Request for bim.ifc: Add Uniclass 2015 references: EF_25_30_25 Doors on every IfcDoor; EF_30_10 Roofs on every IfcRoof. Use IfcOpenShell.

First a look at what the model holds.

```python
import ifcopenshell

model = ifcopenshell.open("bim.ifc")
print(model.schema)
print("classifications:", [c.Name for c in model.by_type("IfcClassification")])
for ifc_class in ("IfcDoor", "IfcRoof", "IfcStair", "IfcWall", "IfcWindow"):
    print(ifc_class, len(model.by_type(ifc_class)))
```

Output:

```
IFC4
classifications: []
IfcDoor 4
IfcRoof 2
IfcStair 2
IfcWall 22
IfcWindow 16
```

```python
import ifcopenshell
import ifcopenshell.api.classification

model = ifcopenshell.open("bim.ifc")

system = ifcopenshell.api.classification.add_classification(model, classification="Uniclass 2015")

codes = {
    "IfcDoor": ("EF_25_30_25", "Doors"),
    "IfcRoof": ("EF_30_10", "Roofs"),
}
for ifc_class, (code, name) in codes.items():
    products = model.by_type(ifc_class)
    ifcopenshell.api.classification.add_reference(
        model, products=products, classification=system, identification=code, name=name
    )
    print(code, len(products))

model.write("bim_rev.ifc")
```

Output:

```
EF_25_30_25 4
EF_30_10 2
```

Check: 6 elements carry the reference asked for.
